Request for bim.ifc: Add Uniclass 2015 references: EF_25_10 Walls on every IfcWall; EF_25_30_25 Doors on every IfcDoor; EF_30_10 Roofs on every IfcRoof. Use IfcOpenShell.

First a look at what the model holds.

```python
import ifcopenshell

model = ifcopenshell.open("bim.ifc")
print(model.schema)
print("classifications:", [c.Name for c in model.by_type("IfcClassification")])
for ifc_class in ("IfcDoor", "IfcRoof", "IfcStair", "IfcWall", "IfcWindow"):
    print(ifc_class, len(model.by_type(ifc_class)))
```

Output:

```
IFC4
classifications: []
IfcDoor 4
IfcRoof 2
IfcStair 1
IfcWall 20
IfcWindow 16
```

```python
import ifcopenshell
import ifcopenshell.api.classification

model = ifcopenshell.open("bim.ifc")

system = ifcopenshell.api.classification.add_classification(model, classification="Uniclass 2015")

codes = {
    "IfcWall": ("EF_25_10", "Walls"),
    "IfcDoor": ("EF_25_30_25", "Doors"),
    "IfcRoof": ("EF_30_10", "Roofs"),
}
for ifc_class, (code, name) in codes.items():
    products = model.by_type(ifc_class)
    ifcopenshell.api.classification.add_reference(
        model, products=products, classification=system, identification=code, name=name
    )
    print(code, len(products))

model.write("bim_updated.ifc")
```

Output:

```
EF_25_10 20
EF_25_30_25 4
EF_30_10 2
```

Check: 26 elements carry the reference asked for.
